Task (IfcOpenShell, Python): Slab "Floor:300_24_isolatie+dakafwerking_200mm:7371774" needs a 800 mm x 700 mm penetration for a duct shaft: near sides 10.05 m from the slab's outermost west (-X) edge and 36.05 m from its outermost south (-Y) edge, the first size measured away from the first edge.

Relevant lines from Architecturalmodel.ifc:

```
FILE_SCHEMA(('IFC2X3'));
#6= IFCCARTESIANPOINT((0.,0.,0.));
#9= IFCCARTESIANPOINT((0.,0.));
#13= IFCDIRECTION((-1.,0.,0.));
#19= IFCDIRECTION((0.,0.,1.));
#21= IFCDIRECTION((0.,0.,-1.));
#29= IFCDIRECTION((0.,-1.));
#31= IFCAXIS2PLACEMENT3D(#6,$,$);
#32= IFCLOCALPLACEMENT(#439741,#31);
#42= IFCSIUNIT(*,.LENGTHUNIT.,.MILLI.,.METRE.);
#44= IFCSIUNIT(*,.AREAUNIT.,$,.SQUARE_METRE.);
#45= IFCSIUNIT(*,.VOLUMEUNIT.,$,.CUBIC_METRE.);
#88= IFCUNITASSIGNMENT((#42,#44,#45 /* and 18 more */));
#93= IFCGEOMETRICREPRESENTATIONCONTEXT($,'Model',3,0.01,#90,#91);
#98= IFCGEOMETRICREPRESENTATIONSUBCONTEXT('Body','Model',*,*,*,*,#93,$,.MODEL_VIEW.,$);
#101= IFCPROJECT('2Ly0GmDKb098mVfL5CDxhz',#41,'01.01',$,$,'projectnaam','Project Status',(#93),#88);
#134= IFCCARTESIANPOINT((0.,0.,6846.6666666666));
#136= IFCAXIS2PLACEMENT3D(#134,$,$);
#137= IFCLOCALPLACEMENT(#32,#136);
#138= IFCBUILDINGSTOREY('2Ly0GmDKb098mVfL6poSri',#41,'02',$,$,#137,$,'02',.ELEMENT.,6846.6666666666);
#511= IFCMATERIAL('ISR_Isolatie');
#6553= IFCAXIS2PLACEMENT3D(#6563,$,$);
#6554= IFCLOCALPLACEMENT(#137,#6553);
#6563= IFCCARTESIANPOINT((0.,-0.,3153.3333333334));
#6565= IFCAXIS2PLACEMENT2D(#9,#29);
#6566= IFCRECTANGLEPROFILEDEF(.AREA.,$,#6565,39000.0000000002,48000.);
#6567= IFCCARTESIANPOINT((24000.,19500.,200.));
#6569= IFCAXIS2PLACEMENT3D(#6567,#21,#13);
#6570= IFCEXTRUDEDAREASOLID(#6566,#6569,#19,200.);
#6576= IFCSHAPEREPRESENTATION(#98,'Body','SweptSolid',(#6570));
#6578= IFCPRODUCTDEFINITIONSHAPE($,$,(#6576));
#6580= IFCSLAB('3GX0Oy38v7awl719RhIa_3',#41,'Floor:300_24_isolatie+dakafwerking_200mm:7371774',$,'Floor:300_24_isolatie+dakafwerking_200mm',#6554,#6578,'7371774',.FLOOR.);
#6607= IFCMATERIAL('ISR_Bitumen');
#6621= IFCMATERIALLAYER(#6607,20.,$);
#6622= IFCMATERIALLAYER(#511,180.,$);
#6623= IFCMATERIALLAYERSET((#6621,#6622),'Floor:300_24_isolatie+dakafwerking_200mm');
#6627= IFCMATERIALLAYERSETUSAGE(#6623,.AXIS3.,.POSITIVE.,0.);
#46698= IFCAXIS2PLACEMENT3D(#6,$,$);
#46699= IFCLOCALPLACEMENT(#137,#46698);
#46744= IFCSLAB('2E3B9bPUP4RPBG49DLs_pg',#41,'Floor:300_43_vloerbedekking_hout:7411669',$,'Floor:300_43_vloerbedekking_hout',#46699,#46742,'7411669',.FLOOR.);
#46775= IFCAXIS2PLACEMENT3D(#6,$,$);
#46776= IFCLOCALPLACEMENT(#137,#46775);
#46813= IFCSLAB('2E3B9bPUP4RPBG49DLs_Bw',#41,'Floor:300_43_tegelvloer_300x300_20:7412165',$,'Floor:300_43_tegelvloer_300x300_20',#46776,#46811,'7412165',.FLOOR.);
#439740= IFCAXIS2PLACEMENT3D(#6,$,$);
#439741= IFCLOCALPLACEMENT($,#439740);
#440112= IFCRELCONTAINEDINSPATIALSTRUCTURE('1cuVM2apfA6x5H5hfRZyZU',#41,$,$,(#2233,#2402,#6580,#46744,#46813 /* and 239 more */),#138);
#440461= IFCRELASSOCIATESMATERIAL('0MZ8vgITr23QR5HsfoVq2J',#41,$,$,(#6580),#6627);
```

```python
import numpy as np
import ifcopenshell
import ifcopenshell.api.feature
import ifcopenshell.api.geometry
import ifcopenshell.api.root
import ifcopenshell.geom
import ifcopenshell.util.placement
import ifcopenshell.util.representation
import ifcopenshell.util.shape
import ifcopenshell.util.unit

model = ifcopenshell.open("Architecturalmodel.ifc")
unit_scale = ifcopenshell.util.unit.calculate_unit_scale(model)
settings = ifcopenshell.geom.settings()


def volume(element):
    """Net volume in cubic metres, openings subtracted."""
    shape = ifcopenshell.geom.create_shape(settings, element)
    return ifcopenshell.util.shape.get_volume(shape.geometry)


slab = model.by_id(6580)
before = volume(slab)

# Extent in the slab's own axes, in metres. The edges named are its -X and -Y sides.
slab_shape = ifcopenshell.geom.create_shape(settings, slab)
vertices = ifcopenshell.util.shape.get_vertices(slab_shape.geometry)
x_min, y_min, bottom = vertices.min(axis=0)
top = vertices[:, 2].max()

opening = ifcopenshell.api.root.create_entity(model, ifc_class="IfcOpeningElement", name="Duct shaft opening")
context = ifcopenshell.util.representation.get_context(model, "Model", "Body", "MODEL_VIEW")
width, depth = 0.8, 0.7
outline = [(0.0, 0.0), (width, 0.0), (width, depth), (0.0, depth), (0.0, 0.0)]
# Overshoot both faces by 50 mm so the cut is clean.
shape = ifcopenshell.api.geometry.add_slab_representation(
    model, context=context, depth=top - bottom + 0.1, polyline=outline
)
ifcopenshell.api.geometry.assign_representation(model, product=opening, representation=shape)

matrix = ifcopenshell.util.placement.get_local_placement(slab.ObjectPlacement)
matrix[:, 3] = matrix @ np.append(np.array([x_min + 10.05, y_min + 36.05, bottom - 0.05]) / unit_scale, 1.0)
ifcopenshell.api.geometry.edit_object_placement(model, product=opening, matrix=matrix, is_si=False)
ifcopenshell.api.feature.add_feature(model, feature=opening, element=slab)

after = volume(slab)

print(f"slab volume {before:.3f} -> {after:.3f} m3")

model.write("Architecturalmodel_edited.ifc")
```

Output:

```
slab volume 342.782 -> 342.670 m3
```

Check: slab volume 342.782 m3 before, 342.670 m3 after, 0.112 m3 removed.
